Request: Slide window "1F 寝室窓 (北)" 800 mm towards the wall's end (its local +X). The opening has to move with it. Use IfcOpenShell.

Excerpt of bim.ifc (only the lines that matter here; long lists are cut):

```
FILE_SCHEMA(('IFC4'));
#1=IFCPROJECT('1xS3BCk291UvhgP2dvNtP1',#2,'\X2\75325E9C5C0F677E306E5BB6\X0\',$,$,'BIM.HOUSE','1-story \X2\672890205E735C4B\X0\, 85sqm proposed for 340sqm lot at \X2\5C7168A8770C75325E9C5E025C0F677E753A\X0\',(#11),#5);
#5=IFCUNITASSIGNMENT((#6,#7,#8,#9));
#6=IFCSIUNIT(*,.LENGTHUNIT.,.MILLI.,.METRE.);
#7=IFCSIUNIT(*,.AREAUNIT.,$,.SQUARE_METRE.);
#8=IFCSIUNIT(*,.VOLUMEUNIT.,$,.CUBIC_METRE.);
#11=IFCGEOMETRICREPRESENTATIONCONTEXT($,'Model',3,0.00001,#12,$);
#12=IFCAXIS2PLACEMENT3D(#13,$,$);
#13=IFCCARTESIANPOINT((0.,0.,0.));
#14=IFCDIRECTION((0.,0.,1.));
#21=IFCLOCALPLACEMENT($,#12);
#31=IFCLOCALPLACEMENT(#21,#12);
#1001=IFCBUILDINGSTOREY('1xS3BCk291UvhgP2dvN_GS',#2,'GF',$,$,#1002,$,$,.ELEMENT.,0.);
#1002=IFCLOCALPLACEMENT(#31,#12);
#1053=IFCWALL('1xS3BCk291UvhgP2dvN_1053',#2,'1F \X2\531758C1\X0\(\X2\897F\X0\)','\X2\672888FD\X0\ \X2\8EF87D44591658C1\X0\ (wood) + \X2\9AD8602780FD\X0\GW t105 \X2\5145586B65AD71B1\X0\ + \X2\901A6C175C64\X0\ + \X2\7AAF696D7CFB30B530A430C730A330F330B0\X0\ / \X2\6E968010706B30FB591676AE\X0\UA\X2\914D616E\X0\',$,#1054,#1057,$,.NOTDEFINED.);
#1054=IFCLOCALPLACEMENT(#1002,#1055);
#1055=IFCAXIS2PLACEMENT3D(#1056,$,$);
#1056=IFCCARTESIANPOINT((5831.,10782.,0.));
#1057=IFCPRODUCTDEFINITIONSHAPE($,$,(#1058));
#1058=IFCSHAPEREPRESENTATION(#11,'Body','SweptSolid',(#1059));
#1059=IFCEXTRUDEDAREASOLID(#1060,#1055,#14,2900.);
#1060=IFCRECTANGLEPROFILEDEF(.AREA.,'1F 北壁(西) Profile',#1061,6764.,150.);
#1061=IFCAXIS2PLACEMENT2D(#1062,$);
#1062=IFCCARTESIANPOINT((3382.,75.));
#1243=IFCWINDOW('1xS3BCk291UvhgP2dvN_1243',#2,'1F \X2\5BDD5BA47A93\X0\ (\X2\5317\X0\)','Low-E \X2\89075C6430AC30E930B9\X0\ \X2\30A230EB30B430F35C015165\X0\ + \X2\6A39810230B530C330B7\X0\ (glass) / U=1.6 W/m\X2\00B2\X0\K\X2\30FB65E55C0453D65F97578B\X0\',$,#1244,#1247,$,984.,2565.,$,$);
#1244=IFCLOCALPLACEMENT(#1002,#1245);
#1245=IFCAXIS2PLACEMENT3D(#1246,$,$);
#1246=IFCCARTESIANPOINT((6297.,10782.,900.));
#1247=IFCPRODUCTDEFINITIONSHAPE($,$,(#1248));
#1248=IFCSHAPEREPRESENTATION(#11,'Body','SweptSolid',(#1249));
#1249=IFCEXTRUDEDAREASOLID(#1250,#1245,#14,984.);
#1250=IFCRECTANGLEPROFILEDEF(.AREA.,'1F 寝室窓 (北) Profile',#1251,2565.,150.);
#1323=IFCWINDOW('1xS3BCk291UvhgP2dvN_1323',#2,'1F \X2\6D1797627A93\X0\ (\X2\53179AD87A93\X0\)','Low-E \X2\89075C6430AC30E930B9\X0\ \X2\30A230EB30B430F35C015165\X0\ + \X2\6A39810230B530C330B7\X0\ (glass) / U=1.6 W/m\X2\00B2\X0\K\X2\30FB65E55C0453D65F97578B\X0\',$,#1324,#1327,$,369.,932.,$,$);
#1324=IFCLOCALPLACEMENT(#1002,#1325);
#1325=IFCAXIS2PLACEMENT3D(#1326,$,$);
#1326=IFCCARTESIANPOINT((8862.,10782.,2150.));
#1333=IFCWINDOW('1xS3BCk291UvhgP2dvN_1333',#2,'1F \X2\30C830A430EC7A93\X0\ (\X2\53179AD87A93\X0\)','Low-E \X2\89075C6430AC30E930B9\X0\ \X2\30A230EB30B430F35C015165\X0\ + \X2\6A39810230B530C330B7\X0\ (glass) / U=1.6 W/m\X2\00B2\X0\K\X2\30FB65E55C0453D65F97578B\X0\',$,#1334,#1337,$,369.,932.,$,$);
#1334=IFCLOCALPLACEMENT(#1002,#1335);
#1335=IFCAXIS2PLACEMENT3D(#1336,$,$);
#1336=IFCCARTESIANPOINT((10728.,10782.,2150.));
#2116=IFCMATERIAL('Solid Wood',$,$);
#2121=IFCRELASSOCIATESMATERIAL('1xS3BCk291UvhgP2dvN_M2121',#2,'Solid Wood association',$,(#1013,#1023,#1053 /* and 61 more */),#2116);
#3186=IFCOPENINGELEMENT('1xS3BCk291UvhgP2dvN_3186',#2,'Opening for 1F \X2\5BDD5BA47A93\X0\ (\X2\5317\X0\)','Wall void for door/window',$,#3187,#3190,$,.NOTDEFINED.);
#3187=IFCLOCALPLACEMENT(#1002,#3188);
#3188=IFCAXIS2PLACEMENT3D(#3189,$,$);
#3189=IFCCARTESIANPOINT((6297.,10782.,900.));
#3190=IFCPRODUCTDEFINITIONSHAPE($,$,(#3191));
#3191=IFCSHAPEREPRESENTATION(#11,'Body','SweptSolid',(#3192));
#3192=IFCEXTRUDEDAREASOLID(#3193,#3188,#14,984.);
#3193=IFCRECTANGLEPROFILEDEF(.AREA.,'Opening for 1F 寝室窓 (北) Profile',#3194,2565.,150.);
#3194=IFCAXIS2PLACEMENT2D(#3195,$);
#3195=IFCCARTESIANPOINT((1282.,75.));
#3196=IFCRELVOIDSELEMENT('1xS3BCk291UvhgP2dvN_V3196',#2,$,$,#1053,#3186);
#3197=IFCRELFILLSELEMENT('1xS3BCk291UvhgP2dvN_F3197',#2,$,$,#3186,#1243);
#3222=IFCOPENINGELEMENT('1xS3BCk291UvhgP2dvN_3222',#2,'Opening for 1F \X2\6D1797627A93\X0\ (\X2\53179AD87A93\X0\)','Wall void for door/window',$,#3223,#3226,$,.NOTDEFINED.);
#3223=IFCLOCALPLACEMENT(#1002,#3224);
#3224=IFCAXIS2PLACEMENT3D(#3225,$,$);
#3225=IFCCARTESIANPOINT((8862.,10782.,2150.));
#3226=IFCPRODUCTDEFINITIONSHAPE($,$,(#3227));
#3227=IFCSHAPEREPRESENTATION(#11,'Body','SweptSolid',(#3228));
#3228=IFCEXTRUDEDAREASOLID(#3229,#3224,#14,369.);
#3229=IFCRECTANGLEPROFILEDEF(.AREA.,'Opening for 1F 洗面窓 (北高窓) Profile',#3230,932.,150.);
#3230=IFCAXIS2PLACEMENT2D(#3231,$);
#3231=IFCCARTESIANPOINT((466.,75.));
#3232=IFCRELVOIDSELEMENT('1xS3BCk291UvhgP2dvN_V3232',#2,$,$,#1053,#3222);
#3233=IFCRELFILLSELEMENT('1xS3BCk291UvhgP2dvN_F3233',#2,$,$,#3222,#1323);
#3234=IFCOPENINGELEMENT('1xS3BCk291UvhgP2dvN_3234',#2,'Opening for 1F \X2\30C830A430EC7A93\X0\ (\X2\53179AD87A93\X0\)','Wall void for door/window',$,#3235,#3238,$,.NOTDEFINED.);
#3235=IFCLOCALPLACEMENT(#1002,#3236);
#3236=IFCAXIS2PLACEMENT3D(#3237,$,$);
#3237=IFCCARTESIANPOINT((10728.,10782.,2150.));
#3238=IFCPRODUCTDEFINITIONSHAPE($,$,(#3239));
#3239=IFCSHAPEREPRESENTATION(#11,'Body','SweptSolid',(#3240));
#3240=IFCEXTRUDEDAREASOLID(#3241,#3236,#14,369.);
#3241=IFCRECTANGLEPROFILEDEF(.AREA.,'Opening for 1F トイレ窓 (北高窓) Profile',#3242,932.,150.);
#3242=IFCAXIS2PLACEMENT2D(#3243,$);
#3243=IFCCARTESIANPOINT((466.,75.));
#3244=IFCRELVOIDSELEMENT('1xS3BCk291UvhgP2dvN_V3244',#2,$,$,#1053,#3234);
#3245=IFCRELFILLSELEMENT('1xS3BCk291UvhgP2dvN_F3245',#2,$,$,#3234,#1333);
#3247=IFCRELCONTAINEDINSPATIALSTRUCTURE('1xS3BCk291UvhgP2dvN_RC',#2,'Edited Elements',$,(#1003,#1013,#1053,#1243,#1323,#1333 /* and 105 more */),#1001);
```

```python
import ifcopenshell
import ifcopenshell.api.geometry
import ifcopenshell.util.placement
import ifcopenshell.util.unit

model = ifcopenshell.open("bim.ifc")
unit_scale = ifcopenshell.util.unit.calculate_unit_scale(model)

window = model.by_guid("1xS3BCk291UvhgP2dvN_1243")
opening = window.FillsVoids[0].RelatingOpeningElement
wall = opening.VoidsElements[0].RelatingBuildingElement

wall_matrix = ifcopenshell.util.placement.get_local_placement(wall.ObjectPlacement)
shift = wall_matrix[:3, 0] * 0.8 / unit_scale
before = ifcopenshell.util.placement.get_local_placement(window.ObjectPlacement)[:3, 3].copy()

# The window is not placed relative to its opening, so move both.
for product in (opening, window):
    matrix = ifcopenshell.util.placement.get_local_placement(product.ObjectPlacement)
    matrix[:3, 3] += shift
    ifcopenshell.api.geometry.edit_object_placement(model, product=product, matrix=matrix, is_si=False)

after = ifcopenshell.util.placement.get_local_placement(window.ObjectPlacement)[:3, 3]
print("window moved by", (after - before).round(3) + 0.0)

model.write("bim_edited.ifc")
```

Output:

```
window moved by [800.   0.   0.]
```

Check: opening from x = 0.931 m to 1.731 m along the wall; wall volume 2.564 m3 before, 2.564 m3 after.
